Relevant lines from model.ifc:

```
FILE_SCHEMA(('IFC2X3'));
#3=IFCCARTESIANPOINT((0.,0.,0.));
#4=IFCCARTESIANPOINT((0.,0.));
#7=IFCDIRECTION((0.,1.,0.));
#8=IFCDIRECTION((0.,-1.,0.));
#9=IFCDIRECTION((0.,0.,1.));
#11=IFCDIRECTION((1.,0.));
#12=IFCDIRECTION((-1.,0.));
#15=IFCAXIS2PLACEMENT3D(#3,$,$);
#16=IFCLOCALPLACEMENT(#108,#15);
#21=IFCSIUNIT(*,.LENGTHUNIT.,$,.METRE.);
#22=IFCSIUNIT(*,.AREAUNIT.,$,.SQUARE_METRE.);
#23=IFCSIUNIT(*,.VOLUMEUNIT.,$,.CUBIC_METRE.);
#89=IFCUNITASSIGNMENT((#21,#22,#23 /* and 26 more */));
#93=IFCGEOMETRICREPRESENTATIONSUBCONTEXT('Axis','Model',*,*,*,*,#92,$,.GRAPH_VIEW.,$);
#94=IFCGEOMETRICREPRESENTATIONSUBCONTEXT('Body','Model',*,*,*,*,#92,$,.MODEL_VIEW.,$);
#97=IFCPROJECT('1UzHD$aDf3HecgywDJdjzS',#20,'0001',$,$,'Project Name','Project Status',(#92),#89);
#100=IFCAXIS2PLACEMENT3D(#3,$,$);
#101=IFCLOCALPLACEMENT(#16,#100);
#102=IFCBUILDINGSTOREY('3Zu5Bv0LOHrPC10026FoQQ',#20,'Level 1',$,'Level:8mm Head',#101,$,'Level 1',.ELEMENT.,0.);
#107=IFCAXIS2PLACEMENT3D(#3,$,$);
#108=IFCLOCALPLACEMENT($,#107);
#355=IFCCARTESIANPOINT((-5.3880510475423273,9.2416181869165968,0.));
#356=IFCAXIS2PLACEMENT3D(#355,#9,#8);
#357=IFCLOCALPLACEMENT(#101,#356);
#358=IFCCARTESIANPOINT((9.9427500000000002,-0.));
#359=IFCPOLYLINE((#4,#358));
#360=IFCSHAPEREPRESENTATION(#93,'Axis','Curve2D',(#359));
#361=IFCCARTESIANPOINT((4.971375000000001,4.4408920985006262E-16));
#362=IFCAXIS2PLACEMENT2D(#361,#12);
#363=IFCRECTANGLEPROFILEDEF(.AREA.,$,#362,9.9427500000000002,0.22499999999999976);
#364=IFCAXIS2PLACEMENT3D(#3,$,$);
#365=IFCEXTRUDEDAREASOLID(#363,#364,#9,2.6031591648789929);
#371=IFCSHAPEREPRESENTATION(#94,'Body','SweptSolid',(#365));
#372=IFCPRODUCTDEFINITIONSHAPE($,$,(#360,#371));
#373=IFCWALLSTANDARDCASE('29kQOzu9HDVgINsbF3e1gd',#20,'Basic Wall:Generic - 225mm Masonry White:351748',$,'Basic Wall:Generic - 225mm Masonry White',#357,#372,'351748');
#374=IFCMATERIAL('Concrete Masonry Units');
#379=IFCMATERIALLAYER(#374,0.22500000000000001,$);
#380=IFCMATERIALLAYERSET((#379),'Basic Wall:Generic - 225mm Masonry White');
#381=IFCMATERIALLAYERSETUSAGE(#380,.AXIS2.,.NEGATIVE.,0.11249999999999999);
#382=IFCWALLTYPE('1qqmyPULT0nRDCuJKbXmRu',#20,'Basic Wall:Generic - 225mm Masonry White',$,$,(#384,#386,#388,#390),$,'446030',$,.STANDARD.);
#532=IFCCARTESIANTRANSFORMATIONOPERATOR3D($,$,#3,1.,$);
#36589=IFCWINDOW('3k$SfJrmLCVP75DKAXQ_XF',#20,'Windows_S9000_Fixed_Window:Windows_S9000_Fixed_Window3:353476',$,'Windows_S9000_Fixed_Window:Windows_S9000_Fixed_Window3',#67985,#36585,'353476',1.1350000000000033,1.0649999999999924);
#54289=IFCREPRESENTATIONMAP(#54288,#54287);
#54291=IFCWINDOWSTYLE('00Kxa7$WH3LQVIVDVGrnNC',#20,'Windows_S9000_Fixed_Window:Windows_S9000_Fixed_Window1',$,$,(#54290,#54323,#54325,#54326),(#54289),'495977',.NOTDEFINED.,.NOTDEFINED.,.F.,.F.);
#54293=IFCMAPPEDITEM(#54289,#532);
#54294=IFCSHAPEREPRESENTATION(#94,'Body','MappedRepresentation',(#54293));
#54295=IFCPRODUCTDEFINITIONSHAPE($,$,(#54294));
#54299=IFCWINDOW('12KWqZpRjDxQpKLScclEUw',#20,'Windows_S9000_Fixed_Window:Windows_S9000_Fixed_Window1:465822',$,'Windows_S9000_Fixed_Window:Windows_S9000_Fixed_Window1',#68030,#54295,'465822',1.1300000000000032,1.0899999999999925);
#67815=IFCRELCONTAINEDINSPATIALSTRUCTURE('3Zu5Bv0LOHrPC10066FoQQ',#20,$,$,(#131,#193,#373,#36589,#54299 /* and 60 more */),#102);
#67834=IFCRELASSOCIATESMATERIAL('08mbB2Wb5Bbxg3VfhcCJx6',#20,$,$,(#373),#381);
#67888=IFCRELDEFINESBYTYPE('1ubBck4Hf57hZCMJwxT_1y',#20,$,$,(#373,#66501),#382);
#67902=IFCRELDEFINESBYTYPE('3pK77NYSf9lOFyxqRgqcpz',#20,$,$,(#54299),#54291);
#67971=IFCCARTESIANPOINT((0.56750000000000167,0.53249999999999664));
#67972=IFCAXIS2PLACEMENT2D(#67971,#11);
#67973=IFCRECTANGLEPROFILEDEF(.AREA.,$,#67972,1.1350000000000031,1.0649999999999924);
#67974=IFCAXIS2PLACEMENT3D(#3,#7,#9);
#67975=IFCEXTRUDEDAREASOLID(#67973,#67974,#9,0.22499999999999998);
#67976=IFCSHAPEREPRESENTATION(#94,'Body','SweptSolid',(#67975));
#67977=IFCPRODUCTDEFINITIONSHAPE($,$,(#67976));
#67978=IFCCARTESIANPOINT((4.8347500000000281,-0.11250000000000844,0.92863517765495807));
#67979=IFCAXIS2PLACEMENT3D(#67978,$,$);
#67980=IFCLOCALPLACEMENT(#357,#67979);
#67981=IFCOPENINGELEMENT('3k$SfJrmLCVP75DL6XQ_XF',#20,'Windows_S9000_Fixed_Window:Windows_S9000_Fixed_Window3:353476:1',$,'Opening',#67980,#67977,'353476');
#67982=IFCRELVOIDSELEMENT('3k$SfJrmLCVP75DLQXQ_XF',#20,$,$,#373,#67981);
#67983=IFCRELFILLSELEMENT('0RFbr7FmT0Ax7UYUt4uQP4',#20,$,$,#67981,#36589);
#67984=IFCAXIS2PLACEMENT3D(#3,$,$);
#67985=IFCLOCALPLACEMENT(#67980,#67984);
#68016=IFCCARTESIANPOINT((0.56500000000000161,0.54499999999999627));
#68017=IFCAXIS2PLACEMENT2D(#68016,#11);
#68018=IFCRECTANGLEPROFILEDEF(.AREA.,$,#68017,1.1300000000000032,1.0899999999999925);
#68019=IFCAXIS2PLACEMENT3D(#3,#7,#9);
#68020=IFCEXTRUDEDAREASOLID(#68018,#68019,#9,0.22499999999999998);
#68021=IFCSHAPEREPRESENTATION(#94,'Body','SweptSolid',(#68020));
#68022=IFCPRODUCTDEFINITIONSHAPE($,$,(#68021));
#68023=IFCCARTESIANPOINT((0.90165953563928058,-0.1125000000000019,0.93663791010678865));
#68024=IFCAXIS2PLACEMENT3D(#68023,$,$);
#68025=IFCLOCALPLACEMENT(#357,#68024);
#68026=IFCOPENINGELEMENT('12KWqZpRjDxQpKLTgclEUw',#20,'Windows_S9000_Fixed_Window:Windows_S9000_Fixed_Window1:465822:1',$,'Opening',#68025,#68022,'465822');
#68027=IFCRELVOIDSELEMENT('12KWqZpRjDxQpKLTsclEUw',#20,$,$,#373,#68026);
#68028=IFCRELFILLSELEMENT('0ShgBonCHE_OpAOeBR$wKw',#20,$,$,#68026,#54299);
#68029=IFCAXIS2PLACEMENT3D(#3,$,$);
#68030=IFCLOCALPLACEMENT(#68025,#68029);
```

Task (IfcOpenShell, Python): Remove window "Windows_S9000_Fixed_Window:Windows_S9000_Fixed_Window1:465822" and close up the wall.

```python
import ifcopenshell
import ifcopenshell.api.feature
import ifcopenshell.api.root
import ifcopenshell.geom
import ifcopenshell.util.shape

model = ifcopenshell.open("model.ifc")
settings = ifcopenshell.geom.settings()


def volume(element):
    """Net volume in cubic metres, openings subtracted."""
    shape = ifcopenshell.geom.create_shape(settings, element)
    return ifcopenshell.util.shape.get_volume(shape.geometry)


window = model.by_guid("12KWqZpRjDxQpKLScclEUw")
opening = window.FillsVoids[0].RelatingOpeningElement
wall = opening.VoidsElements[0].RelatingBuildingElement
before = volume(wall)

ifcopenshell.api.root.remove_product(model, product=window)
ifcopenshell.api.feature.remove_feature(model, feature=opening)

after = volume(wall)

print(f"wall volume {before:.3f} -> {after:.3f} m3")

model.write("model-out.ifc")
```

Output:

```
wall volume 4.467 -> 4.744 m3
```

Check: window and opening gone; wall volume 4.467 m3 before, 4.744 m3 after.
